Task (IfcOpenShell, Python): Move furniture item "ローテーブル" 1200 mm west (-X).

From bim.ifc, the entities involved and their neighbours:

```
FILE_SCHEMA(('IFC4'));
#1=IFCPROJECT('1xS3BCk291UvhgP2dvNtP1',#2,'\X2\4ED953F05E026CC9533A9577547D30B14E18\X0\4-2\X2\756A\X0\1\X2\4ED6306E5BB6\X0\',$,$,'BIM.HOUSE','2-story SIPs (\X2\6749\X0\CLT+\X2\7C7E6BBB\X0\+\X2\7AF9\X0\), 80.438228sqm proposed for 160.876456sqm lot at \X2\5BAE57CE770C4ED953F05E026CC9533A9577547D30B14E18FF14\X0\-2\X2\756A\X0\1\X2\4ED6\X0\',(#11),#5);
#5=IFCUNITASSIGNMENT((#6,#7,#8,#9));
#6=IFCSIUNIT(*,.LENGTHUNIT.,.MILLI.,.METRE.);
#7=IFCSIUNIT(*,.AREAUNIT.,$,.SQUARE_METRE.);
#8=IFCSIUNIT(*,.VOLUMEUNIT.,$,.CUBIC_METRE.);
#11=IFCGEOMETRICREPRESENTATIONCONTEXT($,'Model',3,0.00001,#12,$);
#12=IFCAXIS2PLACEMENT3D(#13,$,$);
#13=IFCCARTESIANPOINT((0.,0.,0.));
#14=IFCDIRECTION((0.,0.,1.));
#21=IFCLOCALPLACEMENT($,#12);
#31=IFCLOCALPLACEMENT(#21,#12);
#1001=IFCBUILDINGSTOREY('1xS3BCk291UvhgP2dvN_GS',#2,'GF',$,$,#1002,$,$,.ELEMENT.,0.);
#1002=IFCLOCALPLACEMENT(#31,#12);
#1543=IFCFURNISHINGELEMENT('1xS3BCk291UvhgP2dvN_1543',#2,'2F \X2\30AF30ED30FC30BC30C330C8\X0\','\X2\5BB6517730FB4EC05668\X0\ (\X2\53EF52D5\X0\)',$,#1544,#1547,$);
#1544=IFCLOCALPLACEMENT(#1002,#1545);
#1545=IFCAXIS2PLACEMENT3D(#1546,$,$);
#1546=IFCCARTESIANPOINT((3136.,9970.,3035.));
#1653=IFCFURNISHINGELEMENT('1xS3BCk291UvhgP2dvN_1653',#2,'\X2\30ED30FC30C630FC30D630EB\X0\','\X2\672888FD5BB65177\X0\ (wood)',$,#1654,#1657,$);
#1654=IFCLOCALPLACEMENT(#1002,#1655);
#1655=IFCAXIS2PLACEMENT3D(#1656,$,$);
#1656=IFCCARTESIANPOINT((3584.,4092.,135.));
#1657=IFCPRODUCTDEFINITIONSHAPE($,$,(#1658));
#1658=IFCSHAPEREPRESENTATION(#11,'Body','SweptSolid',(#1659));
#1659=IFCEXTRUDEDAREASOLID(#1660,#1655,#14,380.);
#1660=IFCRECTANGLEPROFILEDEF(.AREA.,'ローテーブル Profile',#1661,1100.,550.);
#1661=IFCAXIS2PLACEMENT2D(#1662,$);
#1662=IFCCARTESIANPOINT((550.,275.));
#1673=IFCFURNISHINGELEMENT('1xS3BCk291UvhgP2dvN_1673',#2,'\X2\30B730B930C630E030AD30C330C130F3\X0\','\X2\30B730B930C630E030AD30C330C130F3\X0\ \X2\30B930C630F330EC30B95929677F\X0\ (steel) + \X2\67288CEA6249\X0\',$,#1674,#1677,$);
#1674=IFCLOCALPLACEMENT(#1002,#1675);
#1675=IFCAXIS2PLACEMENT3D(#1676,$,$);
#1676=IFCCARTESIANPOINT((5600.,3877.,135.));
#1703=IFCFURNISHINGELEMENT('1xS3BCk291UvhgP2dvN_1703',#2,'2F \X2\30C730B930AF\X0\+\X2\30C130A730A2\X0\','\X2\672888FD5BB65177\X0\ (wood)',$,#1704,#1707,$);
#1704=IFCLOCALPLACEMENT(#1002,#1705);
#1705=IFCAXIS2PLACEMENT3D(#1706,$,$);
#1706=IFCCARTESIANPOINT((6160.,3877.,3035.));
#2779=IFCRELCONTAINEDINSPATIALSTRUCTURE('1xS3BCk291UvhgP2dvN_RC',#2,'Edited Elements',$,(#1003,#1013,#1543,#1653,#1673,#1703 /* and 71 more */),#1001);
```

```python
import ifcopenshell
import ifcopenshell.api.geometry
import ifcopenshell.util.placement

model = ifcopenshell.open("bim.ifc")

item = model.by_guid("1xS3BCk291UvhgP2dvN_1653")
matrix = ifcopenshell.util.placement.get_local_placement(item.ObjectPlacement)
matrix[0, 3] -= 1200.0
ifcopenshell.api.geometry.edit_object_placement(model, product=item, matrix=matrix, is_si=False)

print(ifcopenshell.util.placement.get_local_placement(item.ObjectPlacement).round(3) + 0.0)

model.write("bim_rev.ifc")
```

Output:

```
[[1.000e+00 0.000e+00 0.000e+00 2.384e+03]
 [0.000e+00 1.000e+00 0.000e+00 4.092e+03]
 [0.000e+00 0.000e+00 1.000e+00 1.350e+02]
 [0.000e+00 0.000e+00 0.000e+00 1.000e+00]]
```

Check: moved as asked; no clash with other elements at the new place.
